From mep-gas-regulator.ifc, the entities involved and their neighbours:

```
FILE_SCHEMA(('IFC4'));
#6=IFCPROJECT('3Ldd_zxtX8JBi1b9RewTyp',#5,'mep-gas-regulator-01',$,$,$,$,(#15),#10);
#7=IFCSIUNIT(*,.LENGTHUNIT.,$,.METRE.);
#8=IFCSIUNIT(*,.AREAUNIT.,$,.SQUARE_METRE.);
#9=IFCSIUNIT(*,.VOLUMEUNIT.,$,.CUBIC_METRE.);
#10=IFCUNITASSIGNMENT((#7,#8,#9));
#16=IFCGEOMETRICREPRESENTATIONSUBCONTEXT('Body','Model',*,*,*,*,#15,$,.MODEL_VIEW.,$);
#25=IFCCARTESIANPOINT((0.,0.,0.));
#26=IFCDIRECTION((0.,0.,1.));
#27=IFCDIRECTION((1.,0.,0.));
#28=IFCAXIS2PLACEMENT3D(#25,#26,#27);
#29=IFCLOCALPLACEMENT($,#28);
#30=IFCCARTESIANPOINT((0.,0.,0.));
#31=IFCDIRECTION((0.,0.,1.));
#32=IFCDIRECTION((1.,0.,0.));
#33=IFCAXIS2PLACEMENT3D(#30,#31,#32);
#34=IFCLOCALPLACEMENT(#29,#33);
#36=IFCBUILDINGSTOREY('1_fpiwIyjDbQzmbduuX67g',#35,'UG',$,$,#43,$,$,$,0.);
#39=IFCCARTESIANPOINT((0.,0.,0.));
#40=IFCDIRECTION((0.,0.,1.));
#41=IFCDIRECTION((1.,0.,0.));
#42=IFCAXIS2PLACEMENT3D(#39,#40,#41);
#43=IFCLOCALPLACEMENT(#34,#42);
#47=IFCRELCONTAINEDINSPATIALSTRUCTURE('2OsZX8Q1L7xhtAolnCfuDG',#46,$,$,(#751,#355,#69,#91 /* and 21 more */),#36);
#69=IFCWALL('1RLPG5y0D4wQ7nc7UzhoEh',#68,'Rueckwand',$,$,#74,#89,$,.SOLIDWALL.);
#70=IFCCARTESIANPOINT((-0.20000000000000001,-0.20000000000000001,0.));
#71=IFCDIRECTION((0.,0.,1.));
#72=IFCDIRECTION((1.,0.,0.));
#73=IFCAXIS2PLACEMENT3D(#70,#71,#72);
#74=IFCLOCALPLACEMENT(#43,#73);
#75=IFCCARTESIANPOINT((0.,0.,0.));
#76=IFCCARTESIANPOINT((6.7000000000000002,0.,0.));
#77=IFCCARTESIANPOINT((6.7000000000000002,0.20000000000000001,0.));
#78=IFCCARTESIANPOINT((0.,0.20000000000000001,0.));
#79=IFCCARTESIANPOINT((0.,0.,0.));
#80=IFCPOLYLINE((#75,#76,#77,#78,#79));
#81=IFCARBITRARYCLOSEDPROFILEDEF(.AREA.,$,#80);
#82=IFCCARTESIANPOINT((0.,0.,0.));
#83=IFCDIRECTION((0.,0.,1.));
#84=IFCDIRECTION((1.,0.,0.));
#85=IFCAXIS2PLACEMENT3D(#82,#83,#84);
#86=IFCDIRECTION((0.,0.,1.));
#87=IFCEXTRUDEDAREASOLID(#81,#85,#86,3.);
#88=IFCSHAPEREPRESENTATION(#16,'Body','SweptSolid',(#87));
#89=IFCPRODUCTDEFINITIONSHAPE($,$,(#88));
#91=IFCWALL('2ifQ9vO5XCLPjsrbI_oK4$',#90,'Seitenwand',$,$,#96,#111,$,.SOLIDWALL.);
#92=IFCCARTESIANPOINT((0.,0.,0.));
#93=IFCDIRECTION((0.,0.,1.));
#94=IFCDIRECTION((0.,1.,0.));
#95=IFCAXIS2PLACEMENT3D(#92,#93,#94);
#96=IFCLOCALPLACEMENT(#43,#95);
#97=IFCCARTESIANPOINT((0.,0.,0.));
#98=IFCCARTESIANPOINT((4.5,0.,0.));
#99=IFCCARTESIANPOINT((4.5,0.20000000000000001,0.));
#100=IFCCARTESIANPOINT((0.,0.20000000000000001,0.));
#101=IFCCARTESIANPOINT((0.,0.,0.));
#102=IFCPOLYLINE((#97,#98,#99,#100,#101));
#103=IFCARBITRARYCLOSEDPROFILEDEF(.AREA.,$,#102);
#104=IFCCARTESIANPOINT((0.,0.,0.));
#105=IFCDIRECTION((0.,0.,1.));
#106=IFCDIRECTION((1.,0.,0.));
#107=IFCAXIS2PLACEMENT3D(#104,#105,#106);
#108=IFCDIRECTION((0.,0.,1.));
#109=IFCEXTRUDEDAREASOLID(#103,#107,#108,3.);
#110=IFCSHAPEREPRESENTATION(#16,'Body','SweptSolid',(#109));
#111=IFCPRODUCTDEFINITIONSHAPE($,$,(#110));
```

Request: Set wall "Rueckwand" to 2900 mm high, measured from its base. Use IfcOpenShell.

```python
import ifcopenshell
import ifcopenshell.geom
import ifcopenshell.util.representation
import ifcopenshell.util.shape

model = ifcopenshell.open("mep-gas-regulator.ifc")
settings = ifcopenshell.geom.settings()


def volume(element):
    """Net volume in cubic metres, openings subtracted."""
    shape = ifcopenshell.geom.create_shape(settings, element)
    return ifcopenshell.util.shape.get_volume(shape.geometry)


wall = model.by_guid("1RLPG5y0D4wQ7nc7UzhoEh")
before = volume(wall)

body = ifcopenshell.util.representation.get_representation(wall, "Model", "Body")
solid = body.Items[0]
old_height = solid.Depth
solid.Depth = 2.9
after = volume(wall)

print(f"height {old_height:g} -> {solid.Depth:g}, volume {before:.3f} -> {after:.3f} m3")

model.write("mep-gas-regulator_edited.ifc")
```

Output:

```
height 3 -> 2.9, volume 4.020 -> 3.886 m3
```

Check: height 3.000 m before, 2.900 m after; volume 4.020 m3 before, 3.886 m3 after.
